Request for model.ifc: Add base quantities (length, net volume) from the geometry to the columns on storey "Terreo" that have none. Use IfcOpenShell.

First a look at what the model holds.

```python
import ifcopenshell
import ifcopenshell.util.element
import ifcopenshell.util.unit

model = ifcopenshell.open("model.ifc")
print(model.schema)
for unit_type in ("LENGTHUNIT", "AREAUNIT", "VOLUMEUNIT"):
    print(unit_type, ifcopenshell.util.unit.calculate_unit_scale(model, unit_type))
storey = next(s for s in model.by_type("IfcBuildingStorey") if s.Name == "Terreo")
columns = [e for e in ifcopenshell.util.element.get_decomposition(storey) if e.is_a("IfcColumn")]
for e in sorted(columns, key=lambda e: e.id()):
    print(e.id(), e.is_a(), e.Name, list(ifcopenshell.util.element.get_psets(e, qtos_only=True)), sep=" | ")
```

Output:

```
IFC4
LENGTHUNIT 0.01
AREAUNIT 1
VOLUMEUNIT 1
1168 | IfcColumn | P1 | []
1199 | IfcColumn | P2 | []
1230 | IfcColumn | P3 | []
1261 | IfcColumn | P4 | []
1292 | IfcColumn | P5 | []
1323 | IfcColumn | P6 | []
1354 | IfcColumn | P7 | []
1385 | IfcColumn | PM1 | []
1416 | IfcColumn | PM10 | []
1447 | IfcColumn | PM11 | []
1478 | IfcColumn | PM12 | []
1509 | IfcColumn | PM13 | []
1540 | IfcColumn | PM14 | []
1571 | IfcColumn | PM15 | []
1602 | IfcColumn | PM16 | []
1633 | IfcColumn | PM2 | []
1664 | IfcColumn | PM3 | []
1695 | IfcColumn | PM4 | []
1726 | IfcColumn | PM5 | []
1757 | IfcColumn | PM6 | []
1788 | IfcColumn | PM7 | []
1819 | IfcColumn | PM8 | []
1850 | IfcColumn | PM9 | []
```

```python
import ifcopenshell
import ifcopenshell.api.pset
import ifcopenshell.geom
import ifcopenshell.util.element
import ifcopenshell.util.shape
import ifcopenshell.util.unit

model = ifcopenshell.open("model.ifc")
unit_scale = ifcopenshell.util.unit.calculate_unit_scale(model)
volume_scale = ifcopenshell.util.unit.calculate_unit_scale(model, "VOLUMEUNIT")
settings = ifcopenshell.geom.settings()

storey = next(s for s in model.by_type("IfcBuildingStorey") if s.Name == "Terreo")
columns = [e for e in ifcopenshell.util.element.get_decomposition(storey) if e.is_a("IfcColumn")]

for e in sorted(columns, key=lambda e: e.id()):
    if ifcopenshell.util.element.get_psets(e, qtos_only=True, should_inherit=False):
        continue
    # Geometry comes back in metres, in the element's own axes.
    shape = ifcopenshell.geom.create_shape(settings, e)
    values = {
        "Length": ifcopenshell.util.shape.get_z(shape.geometry) / unit_scale,
        "NetVolume": ifcopenshell.util.shape.get_volume(shape.geometry) / volume_scale,
    }
    qto = ifcopenshell.api.pset.add_qto(model, product=e, name="Qto_ColumnBaseQuantities")
    ifcopenshell.api.pset.edit_qto(model, qto=qto, properties=values)
    print(e.id(), {k: round(v, 3) for k, v in values.items()})

model.write("model-out.ifc")
```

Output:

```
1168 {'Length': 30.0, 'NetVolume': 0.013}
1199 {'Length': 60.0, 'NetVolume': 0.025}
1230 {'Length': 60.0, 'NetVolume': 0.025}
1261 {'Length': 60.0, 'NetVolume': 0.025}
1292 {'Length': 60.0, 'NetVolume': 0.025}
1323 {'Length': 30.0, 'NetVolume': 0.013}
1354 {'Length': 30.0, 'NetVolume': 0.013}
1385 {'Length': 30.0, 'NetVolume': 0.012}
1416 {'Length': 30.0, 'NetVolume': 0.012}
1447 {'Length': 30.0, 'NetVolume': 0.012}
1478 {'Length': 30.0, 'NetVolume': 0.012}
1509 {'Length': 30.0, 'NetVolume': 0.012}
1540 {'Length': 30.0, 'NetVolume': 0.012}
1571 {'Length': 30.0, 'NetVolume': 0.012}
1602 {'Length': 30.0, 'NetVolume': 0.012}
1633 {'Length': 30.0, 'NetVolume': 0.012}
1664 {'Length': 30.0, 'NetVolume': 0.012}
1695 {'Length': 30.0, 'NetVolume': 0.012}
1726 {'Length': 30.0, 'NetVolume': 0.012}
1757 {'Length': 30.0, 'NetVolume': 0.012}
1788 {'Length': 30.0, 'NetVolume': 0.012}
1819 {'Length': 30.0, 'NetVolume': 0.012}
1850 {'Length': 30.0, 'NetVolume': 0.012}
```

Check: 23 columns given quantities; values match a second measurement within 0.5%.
